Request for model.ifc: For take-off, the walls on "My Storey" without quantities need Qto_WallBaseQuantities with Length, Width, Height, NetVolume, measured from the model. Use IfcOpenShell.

First a look at what the model holds.

```python
import ifcopenshell
import ifcopenshell.util.element
import ifcopenshell.util.unit

model = ifcopenshell.open("model.ifc")
print(model.schema)
for unit_type in ("LENGTHUNIT", "AREAUNIT", "VOLUMEUNIT"):
    print(unit_type, ifcopenshell.util.unit.calculate_unit_scale(model, unit_type))
storey = next(s for s in model.by_type("IfcBuildingStorey") if s.Name == "My Storey")
walls = [e for e in ifcopenshell.util.element.get_decomposition(storey) if e.is_a("IfcWall")]
for e in sorted(walls, key=lambda e: e.id()):
    print(e.id(), e.is_a(), e.Name, list(ifcopenshell.util.element.get_psets(e, qtos_only=True)), sep=" | ")
```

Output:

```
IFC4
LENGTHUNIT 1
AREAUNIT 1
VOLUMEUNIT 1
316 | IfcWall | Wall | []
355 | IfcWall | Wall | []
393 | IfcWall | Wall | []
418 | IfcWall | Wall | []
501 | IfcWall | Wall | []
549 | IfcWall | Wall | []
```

```python
import ifcopenshell
import ifcopenshell.api.pset
import ifcopenshell.geom
import ifcopenshell.util.element
import ifcopenshell.util.shape
import ifcopenshell.util.unit

model = ifcopenshell.open("model.ifc")
unit_scale = ifcopenshell.util.unit.calculate_unit_scale(model)
volume_scale = ifcopenshell.util.unit.calculate_unit_scale(model, "VOLUMEUNIT")
settings = ifcopenshell.geom.settings()

storey = next(s for s in model.by_type("IfcBuildingStorey") if s.Name == "My Storey")
walls = [e for e in ifcopenshell.util.element.get_decomposition(storey) if e.is_a("IfcWall")]

for e in sorted(walls, key=lambda e: e.id()):
    if ifcopenshell.util.element.get_psets(e, qtos_only=True, should_inherit=False):
        continue
    # Geometry comes back in metres, in the element's own axes.
    shape = ifcopenshell.geom.create_shape(settings, e)
    values = {
        "Length": ifcopenshell.util.shape.get_x(shape.geometry) / unit_scale,
        "Width": ifcopenshell.util.shape.get_y(shape.geometry) / unit_scale,
        "Height": ifcopenshell.util.shape.get_z(shape.geometry) / unit_scale,
        "NetVolume": ifcopenshell.util.shape.get_volume(shape.geometry) / volume_scale,
    }
    qto = ifcopenshell.api.pset.add_qto(model, product=e, name="Qto_WallBaseQuantities")
    ifcopenshell.api.pset.edit_qto(model, qto=qto, properties=values)
    print(e.id(), {k: round(v, 3) for k, v in values.items()})

model.write("model_updated.ifc")
```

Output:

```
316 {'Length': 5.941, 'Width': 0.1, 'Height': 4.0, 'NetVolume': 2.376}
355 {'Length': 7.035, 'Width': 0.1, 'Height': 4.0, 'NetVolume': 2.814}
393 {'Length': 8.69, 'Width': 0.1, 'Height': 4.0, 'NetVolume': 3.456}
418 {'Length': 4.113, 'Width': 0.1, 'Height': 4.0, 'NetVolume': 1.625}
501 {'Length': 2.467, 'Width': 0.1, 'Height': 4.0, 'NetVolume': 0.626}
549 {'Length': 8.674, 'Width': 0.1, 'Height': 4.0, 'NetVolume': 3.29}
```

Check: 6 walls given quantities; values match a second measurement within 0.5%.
